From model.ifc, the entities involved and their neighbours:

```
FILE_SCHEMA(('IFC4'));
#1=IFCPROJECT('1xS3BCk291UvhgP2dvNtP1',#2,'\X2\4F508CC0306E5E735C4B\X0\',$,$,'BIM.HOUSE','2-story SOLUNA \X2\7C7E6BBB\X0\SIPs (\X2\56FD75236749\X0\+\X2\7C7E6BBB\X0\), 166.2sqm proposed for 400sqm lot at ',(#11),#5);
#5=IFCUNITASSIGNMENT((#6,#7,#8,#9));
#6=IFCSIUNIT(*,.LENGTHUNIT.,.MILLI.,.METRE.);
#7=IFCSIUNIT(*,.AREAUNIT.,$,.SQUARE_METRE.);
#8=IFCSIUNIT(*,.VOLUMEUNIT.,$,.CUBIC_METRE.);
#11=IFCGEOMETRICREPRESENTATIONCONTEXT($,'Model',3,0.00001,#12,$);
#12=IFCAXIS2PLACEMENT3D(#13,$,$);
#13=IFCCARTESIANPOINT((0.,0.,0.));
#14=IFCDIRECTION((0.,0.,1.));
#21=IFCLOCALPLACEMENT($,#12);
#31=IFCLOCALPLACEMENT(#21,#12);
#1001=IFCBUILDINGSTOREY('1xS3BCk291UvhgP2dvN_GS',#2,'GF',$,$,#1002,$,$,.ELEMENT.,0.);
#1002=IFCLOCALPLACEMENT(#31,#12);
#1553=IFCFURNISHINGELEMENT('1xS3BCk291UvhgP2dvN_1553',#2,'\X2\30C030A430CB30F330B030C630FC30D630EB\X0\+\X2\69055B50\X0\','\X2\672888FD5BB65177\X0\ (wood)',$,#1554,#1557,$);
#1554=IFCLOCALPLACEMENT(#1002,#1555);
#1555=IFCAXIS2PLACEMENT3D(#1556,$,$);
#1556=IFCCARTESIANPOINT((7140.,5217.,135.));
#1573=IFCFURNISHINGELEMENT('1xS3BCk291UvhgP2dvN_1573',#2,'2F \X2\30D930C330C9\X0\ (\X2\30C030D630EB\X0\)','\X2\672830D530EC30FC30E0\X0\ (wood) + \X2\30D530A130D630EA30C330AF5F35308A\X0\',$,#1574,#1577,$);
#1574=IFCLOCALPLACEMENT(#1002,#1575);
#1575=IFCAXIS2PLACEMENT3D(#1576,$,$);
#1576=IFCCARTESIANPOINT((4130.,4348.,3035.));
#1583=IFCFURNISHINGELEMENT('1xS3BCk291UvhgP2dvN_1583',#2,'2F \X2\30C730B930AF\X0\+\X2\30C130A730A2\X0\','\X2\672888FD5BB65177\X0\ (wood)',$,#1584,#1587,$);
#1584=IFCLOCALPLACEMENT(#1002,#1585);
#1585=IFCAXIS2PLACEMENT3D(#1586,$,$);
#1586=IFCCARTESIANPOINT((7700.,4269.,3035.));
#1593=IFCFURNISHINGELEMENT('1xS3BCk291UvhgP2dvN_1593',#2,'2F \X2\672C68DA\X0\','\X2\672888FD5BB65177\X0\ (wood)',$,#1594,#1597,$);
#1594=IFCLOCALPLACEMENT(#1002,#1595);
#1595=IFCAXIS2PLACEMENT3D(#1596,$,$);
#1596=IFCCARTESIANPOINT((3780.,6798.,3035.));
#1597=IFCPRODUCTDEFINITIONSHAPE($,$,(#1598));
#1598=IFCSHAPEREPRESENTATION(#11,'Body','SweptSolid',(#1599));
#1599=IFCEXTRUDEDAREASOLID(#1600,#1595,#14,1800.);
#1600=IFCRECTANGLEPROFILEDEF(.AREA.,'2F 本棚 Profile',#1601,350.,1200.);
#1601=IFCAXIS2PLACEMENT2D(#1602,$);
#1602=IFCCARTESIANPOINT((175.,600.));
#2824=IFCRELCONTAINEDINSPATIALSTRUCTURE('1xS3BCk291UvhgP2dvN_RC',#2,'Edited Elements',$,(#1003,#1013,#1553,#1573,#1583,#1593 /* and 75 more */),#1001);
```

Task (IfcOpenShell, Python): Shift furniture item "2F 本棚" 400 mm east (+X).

```python
import ifcopenshell
import ifcopenshell.api.geometry
import ifcopenshell.util.placement
import ifcopenshell.util.unit

model = ifcopenshell.open("model.ifc")
unit_scale = ifcopenshell.util.unit.calculate_unit_scale(model)

item = model.by_guid("1xS3BCk291UvhgP2dvN_1593")
matrix = ifcopenshell.util.placement.get_local_placement(item.ObjectPlacement)
matrix[0, 3] += 0.4 / unit_scale
ifcopenshell.api.geometry.edit_object_placement(model, product=item, matrix=matrix, is_si=False)

print(ifcopenshell.util.placement.get_local_placement(item.ObjectPlacement).round(3) + 0.0)

model.write("model_rev.ifc")
```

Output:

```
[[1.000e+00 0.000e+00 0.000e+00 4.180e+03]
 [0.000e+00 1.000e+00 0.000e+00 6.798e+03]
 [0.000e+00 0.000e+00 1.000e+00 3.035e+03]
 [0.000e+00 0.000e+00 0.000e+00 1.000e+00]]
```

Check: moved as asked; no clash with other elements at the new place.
